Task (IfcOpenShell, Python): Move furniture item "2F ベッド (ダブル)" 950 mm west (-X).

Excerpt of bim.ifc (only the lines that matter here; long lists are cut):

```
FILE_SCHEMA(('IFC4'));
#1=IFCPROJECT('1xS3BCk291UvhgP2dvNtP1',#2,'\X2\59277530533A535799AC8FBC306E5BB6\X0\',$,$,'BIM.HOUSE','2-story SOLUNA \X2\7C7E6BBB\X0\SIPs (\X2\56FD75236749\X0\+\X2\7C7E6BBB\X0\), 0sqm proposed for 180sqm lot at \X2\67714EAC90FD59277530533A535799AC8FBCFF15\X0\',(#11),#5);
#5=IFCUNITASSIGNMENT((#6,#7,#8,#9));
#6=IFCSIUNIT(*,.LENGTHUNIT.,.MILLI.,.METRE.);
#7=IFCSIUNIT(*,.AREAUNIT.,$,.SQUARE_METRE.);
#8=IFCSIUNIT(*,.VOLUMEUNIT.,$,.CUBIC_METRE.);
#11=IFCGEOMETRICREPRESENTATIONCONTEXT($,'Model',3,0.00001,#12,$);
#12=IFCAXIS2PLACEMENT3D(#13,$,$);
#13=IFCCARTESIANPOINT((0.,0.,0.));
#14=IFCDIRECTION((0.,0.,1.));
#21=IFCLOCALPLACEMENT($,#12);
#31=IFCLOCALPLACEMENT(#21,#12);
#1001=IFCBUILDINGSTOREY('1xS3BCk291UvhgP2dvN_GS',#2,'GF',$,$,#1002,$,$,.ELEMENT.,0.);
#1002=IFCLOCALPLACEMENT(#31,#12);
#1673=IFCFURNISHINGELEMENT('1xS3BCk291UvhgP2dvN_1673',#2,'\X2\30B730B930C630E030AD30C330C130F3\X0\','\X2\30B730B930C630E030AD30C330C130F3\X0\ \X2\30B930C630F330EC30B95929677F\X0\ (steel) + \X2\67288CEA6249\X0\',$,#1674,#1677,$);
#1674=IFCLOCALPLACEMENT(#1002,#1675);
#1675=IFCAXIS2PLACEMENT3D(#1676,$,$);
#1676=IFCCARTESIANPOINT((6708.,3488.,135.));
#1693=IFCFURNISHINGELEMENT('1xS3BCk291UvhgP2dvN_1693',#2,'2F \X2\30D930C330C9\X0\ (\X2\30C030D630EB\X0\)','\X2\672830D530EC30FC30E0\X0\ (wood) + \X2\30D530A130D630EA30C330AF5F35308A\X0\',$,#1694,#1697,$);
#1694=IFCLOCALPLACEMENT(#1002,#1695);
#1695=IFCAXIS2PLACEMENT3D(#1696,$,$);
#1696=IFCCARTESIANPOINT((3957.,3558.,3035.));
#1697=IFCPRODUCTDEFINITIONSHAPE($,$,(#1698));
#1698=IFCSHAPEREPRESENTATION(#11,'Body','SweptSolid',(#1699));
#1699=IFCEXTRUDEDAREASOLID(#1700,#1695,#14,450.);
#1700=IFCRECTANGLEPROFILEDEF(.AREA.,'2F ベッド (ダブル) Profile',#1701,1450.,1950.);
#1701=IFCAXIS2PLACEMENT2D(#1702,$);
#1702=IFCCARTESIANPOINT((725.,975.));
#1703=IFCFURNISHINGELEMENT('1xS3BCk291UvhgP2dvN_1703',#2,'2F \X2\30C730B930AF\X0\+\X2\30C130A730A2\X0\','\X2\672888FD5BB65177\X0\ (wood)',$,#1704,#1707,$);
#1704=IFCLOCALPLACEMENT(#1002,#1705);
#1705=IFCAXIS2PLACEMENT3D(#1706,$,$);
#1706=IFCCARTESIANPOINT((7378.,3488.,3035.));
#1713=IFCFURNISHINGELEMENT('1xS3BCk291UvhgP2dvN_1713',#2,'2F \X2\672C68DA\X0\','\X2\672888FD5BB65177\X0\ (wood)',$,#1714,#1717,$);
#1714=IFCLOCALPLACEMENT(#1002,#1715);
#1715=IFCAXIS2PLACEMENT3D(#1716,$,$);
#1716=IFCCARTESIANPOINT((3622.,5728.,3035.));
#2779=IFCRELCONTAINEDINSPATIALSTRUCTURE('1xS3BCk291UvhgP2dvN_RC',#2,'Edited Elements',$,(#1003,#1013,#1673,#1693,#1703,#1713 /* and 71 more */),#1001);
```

```python
import ifcopenshell
import ifcopenshell.api.geometry
import ifcopenshell.util.placement
import ifcopenshell.util.unit

model = ifcopenshell.open("bim.ifc")
unit_scale = ifcopenshell.util.unit.calculate_unit_scale(model)

item = model.by_guid("1xS3BCk291UvhgP2dvN_1693")
matrix = ifcopenshell.util.placement.get_local_placement(item.ObjectPlacement)
matrix[0, 3] -= 0.95 / unit_scale
ifcopenshell.api.geometry.edit_object_placement(model, product=item, matrix=matrix, is_si=False)

print(ifcopenshell.util.placement.get_local_placement(item.ObjectPlacement).round(3) + 0.0)

model.write("bim_v2.ifc")
```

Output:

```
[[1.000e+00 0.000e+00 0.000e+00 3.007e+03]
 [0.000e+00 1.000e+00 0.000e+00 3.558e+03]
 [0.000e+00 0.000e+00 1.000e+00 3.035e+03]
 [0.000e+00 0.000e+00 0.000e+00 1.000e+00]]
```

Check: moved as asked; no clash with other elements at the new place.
